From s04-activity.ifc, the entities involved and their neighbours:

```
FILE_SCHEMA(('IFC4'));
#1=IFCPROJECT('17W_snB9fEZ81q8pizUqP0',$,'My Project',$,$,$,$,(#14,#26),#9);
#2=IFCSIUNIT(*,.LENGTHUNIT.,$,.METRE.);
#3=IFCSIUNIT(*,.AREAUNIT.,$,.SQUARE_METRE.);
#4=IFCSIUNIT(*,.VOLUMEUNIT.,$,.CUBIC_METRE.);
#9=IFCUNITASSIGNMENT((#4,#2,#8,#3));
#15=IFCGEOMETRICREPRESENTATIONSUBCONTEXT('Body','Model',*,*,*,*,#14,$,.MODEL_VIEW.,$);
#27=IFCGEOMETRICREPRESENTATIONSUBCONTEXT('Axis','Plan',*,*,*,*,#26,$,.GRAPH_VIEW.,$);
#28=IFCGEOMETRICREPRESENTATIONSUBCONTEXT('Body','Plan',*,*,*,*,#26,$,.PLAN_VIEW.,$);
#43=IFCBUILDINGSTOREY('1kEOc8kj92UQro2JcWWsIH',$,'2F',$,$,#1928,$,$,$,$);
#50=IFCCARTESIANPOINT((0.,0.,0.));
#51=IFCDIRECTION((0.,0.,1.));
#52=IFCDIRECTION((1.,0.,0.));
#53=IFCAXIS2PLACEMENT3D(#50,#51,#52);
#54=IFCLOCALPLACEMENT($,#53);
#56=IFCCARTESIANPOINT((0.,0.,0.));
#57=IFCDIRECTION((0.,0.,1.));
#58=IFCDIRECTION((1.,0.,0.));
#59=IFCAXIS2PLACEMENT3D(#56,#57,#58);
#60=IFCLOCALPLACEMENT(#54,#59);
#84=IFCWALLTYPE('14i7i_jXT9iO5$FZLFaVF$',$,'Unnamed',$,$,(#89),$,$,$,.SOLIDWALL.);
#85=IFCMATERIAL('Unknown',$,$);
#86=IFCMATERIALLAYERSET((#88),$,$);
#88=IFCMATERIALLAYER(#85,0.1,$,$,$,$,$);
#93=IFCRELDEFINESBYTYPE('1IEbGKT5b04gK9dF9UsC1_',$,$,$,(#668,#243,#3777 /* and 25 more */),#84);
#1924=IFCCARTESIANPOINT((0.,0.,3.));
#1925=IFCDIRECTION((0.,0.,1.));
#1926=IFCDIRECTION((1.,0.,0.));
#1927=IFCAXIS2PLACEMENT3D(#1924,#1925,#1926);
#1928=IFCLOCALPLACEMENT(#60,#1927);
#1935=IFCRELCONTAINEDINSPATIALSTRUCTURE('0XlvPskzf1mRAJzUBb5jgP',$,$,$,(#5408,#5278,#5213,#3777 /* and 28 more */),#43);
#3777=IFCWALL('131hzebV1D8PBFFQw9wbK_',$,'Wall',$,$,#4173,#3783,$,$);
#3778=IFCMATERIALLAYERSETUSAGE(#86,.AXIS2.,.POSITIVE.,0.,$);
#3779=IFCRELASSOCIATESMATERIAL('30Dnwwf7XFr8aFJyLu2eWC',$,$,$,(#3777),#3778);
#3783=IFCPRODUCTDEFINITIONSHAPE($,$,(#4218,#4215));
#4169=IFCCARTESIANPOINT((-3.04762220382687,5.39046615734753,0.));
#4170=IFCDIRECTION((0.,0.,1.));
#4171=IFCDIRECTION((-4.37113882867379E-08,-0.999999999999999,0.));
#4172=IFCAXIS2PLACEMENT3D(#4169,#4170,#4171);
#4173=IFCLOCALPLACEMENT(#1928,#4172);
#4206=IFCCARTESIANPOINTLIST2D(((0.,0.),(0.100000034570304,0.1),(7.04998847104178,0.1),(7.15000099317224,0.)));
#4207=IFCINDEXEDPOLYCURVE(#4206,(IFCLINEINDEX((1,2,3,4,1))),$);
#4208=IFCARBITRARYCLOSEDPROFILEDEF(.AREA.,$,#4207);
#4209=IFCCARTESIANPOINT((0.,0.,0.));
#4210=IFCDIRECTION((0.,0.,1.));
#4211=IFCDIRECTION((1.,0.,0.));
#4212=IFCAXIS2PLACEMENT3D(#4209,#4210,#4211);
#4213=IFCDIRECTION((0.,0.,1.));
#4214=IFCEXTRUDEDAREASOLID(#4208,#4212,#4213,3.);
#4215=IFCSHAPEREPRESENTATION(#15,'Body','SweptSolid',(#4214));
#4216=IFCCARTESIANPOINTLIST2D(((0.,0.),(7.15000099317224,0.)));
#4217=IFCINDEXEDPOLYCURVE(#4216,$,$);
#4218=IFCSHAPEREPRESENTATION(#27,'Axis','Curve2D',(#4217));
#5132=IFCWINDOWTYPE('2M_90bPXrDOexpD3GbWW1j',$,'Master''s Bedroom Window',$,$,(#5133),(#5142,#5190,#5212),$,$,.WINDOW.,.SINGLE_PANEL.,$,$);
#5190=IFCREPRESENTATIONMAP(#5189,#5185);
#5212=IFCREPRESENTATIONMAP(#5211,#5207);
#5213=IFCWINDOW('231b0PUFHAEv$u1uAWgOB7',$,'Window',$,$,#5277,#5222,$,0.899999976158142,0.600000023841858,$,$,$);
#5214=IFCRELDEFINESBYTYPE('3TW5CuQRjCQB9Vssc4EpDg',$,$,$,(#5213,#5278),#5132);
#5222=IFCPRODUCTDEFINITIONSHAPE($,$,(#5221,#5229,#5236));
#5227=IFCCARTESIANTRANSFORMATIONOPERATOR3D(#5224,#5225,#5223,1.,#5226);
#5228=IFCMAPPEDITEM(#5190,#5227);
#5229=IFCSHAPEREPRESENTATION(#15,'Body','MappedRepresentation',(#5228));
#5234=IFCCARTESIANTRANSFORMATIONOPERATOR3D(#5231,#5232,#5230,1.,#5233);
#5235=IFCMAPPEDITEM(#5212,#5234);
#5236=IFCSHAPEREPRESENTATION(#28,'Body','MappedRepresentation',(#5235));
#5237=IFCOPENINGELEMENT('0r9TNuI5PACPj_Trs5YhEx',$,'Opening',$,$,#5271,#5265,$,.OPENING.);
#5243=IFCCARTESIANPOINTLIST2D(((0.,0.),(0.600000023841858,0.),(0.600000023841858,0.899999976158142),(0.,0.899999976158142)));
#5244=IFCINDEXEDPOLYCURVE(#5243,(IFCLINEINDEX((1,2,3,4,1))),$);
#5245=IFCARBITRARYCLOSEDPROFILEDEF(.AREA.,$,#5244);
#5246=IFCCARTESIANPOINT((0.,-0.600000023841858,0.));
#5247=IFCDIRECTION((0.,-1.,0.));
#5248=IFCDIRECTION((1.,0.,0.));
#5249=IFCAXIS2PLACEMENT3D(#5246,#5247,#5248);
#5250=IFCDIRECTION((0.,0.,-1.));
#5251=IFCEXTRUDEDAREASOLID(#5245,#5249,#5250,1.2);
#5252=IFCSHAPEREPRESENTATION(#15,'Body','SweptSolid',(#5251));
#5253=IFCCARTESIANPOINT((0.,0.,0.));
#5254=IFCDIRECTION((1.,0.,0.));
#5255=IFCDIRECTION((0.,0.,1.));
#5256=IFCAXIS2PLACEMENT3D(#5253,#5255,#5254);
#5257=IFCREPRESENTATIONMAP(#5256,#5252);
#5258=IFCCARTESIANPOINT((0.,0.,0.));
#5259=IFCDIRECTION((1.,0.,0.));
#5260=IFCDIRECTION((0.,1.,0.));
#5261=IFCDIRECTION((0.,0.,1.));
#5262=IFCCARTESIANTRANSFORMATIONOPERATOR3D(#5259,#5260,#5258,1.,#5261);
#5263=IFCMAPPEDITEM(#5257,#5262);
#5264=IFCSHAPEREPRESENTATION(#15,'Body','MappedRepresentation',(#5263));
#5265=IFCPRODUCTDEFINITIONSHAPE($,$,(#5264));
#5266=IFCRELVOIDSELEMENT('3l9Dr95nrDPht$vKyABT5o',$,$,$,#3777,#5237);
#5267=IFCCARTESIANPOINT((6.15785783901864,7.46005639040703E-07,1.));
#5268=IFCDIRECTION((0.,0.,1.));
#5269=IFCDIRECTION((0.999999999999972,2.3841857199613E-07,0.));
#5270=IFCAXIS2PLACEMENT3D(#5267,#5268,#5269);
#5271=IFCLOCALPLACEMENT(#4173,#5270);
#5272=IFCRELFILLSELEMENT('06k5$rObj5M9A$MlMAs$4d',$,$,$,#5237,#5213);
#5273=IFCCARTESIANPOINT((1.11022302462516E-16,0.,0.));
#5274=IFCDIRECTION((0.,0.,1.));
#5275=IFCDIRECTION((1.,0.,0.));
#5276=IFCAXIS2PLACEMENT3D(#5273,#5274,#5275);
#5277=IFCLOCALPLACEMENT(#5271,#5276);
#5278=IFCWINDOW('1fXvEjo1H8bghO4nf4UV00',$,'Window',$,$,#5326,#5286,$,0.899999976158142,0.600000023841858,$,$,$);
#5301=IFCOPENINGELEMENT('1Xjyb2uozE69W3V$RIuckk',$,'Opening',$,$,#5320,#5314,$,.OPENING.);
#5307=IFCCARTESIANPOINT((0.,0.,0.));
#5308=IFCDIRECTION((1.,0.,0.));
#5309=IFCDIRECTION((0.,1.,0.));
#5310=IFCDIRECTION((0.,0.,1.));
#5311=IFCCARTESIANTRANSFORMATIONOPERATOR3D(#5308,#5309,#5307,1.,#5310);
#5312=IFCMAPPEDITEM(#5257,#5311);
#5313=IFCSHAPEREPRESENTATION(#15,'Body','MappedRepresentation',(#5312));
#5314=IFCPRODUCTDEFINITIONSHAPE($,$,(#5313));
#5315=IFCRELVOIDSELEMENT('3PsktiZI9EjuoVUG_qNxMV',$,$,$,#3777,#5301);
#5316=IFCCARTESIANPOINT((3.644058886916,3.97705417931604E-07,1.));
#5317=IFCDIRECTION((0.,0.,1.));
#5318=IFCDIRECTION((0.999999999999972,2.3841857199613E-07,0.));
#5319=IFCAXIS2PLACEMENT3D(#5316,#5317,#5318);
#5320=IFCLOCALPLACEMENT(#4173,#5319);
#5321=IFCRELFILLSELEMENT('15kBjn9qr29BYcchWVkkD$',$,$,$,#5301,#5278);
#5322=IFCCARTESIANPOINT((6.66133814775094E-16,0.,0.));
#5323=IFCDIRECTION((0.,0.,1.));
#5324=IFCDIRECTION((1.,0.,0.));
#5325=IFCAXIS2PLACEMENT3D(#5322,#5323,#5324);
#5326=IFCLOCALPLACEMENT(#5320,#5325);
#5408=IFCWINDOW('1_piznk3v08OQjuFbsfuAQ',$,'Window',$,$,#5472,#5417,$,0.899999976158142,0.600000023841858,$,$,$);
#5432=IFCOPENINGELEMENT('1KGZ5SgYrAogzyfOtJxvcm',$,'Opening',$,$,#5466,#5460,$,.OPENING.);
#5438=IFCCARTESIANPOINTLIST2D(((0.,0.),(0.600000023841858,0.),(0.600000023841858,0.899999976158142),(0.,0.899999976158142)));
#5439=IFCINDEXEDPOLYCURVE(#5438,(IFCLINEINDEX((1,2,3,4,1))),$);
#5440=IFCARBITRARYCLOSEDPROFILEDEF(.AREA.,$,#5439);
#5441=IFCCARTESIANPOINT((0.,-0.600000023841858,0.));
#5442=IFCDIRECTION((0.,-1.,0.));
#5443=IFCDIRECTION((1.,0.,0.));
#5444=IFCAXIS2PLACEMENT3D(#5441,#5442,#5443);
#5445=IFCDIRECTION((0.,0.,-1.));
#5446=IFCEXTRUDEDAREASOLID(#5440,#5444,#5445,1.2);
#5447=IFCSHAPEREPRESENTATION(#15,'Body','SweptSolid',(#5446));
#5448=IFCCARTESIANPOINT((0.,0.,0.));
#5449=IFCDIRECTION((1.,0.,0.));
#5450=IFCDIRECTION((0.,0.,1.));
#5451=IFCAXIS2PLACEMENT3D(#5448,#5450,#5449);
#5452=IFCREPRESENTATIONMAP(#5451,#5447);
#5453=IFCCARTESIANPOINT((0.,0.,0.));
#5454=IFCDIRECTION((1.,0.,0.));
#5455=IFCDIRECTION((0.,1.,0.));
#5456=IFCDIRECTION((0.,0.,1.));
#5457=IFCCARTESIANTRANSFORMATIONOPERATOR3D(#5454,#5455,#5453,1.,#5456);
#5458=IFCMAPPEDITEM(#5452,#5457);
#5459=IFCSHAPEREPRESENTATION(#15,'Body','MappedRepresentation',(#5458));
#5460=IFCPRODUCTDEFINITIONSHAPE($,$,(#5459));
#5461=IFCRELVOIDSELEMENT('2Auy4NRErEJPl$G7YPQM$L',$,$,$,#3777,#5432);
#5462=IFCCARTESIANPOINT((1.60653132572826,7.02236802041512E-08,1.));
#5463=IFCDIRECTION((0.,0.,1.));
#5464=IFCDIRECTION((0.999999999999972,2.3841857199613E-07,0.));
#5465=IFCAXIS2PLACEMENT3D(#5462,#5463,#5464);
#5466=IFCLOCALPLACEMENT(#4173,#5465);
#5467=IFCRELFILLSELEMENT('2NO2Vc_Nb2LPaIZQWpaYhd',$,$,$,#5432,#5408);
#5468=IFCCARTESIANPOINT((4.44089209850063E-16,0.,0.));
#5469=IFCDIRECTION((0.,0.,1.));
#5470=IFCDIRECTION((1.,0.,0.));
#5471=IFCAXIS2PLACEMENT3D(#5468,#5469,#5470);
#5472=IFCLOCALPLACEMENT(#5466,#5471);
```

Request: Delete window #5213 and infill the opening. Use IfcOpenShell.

```python
import ifcopenshell
import ifcopenshell.api.feature
import ifcopenshell.api.root
import ifcopenshell.geom
import ifcopenshell.util.shape

model = ifcopenshell.open("s04-activity.ifc")
settings = ifcopenshell.geom.settings()


def volume(element):
    """Net volume in cubic metres, openings subtracted."""
    shape = ifcopenshell.geom.create_shape(settings, element)
    return ifcopenshell.util.shape.get_volume(shape.geometry)


window = model.by_id(5213)
opening = window.FillsVoids[0].RelatingOpeningElement
wall = opening.VoidsElements[0].RelatingBuildingElement
before = volume(wall)

ifcopenshell.api.root.remove_product(model, product=window)
ifcopenshell.api.feature.remove_feature(model, feature=opening)

after = volume(wall)

print(f"wall volume {before:.3f} -> {after:.3f} m3")

model.write("s04-activity-out.ifc")
```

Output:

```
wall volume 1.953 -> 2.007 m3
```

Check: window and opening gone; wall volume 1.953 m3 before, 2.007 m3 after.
